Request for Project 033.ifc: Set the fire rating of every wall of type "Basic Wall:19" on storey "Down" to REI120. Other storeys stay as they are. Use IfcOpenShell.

First a look at what the model holds.

```python
import ifcopenshell
import ifcopenshell.util.element

model = ifcopenshell.open("Project 033.ifc")
print(model.schema)
storey = next(s for s in model.by_type("IfcBuildingStorey") if s.Name == "Down")
walls = [e for e in ifcopenshell.util.element.get_decomposition(storey) if e.is_a("IfcWall")]
seen = {}
for e in walls:
    element_type = ifcopenshell.util.element.get_type(e)
    key = (element_type.Name if element_type != e and element_type else None, ifcopenshell.util.element.get_pset(e, "Pset_WallCommon", "FireRating"))
    seen[key] = seen.get(key, 0) + 1
for (name, value), count in sorted(seen.items(), key=str):
    print(count, "x", name, "|", value)
```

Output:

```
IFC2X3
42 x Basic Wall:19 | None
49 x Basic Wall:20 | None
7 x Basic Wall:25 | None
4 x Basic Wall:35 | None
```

```python
import ifcopenshell
import ifcopenshell.api.pset
import ifcopenshell.util.element

model = ifcopenshell.open("Project 033.ifc")

storey = next(s for s in model.by_type("IfcBuildingStorey") if s.Name == "Down")
walls = [e for e in ifcopenshell.util.element.get_decomposition(storey) if e.is_a("IfcWall")]

count = 0
for e in walls:
    element_type = ifcopenshell.util.element.get_type(e)
    if element_type in (None, e) or element_type.Name != "Basic Wall:19":
        continue
    # add_pset returns the element's existing set when there is one.
    pset = ifcopenshell.api.pset.add_pset(model, product=e, name="Pset_WallCommon")
    ifcopenshell.api.pset.edit_pset(model, pset=pset, properties={"FireRating": "REI120"})
    count += 1

print(count, "walls updated")

model.write("Project 033_rev.ifc")
```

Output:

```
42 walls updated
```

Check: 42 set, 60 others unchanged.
